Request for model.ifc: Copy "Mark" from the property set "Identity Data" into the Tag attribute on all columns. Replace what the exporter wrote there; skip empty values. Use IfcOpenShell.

First a look at what the model holds.

```python
import ifcopenshell
import ifcopenshell.util.element

model = ifcopenshell.open("model.ifc")
print(model.schema)
columns = model.by_type("IfcColumn")
print(len(columns), "columns")
for e in columns[:8]:
    source = ifcopenshell.util.element.get_pset(e, "Identity Data", "Mark")
    target = e.Tag
    print(e.id(), repr(source), repr(target), sep=" | ")
```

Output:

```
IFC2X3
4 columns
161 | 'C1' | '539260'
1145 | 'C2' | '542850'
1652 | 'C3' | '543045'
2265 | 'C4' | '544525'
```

```python
import ifcopenshell
import ifcopenshell.util.element

model = ifcopenshell.open("model.ifc")

count = 0
for e in model.by_type("IfcColumn"):
    value = ifcopenshell.util.element.get_pset(e, "Identity Data", "Mark")
    current = e.Tag
    if not value or not value.strip() or current == value:
        continue
    e.Tag = value
    count += 1

print(count, "columns updated")

model.write("model_v2.ifc")
```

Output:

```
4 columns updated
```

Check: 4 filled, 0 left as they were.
